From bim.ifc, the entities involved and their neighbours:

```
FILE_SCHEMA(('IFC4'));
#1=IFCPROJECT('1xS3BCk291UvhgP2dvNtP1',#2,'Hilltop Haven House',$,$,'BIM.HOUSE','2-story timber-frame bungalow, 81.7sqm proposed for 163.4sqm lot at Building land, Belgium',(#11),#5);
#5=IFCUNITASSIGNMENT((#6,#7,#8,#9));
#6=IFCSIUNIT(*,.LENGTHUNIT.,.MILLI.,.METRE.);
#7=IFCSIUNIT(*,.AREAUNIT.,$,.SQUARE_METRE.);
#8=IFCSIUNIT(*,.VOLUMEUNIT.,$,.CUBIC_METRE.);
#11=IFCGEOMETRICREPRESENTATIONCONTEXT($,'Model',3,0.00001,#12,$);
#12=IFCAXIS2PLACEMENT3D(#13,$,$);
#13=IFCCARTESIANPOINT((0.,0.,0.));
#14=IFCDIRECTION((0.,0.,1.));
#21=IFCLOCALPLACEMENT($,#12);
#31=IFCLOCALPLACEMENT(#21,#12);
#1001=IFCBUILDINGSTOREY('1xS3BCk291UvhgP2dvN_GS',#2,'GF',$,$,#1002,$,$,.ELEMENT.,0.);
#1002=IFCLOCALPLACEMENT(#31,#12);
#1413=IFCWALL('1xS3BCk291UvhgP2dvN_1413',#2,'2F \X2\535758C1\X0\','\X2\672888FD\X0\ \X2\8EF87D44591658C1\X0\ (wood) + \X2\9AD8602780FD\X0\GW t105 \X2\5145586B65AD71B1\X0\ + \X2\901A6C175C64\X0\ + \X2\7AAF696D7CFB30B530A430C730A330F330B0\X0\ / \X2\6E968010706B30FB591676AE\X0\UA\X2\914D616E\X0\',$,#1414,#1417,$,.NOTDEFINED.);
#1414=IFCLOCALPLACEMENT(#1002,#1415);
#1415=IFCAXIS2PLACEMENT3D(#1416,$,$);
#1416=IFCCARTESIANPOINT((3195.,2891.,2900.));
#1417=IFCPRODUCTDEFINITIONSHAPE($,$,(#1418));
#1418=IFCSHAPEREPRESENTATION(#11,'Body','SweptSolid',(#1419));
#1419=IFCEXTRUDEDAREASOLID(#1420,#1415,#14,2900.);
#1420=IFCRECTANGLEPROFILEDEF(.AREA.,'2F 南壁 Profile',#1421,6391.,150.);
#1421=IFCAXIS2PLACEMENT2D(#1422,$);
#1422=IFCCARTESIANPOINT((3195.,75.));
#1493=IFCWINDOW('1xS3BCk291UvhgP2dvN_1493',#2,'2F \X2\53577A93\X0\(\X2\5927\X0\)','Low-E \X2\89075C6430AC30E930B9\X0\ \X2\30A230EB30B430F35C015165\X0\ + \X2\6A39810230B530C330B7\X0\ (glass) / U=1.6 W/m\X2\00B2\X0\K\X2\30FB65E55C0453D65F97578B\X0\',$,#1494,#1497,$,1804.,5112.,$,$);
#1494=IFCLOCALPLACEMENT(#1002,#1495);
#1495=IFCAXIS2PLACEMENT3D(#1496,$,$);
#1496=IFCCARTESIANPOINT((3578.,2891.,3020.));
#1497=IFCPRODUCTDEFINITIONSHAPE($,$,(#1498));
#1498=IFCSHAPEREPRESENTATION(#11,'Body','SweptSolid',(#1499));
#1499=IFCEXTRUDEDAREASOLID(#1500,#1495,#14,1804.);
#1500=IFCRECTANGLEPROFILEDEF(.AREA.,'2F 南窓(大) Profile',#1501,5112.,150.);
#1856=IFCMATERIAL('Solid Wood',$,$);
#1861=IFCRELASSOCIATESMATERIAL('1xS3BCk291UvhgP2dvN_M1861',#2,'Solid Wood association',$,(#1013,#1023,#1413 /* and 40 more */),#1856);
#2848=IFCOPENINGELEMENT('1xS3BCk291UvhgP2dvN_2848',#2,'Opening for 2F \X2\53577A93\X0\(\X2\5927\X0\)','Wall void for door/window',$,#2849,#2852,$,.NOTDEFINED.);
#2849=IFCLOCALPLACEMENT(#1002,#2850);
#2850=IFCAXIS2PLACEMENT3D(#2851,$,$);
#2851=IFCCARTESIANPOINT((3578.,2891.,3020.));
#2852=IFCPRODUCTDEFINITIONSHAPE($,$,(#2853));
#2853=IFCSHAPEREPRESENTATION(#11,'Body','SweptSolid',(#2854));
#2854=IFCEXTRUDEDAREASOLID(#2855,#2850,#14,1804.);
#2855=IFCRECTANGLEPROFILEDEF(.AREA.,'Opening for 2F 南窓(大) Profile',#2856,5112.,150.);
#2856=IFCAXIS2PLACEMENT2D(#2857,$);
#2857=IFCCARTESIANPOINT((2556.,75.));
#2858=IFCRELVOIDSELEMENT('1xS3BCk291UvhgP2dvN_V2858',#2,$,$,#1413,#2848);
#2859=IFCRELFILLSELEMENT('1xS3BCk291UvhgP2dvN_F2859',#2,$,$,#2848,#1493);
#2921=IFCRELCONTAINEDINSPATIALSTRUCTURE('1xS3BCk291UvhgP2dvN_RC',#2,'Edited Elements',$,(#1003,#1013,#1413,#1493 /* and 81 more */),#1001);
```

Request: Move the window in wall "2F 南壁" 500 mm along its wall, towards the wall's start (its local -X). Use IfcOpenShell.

```python
import ifcopenshell
import ifcopenshell.api.geometry
import ifcopenshell.util.placement

model = ifcopenshell.open("bim.ifc")

window = model.by_guid("1xS3BCk291UvhgP2dvN_1493")
opening = window.FillsVoids[0].RelatingOpeningElement
wall = opening.VoidsElements[0].RelatingBuildingElement

wall_matrix = ifcopenshell.util.placement.get_local_placement(wall.ObjectPlacement)
shift = wall_matrix[:3, 0] * -500.0
before = ifcopenshell.util.placement.get_local_placement(window.ObjectPlacement)[:3, 3].copy()

# The window is not placed relative to its opening, so move both.
for product in (opening, window):
    matrix = ifcopenshell.util.placement.get_local_placement(product.ObjectPlacement)
    matrix[:3, 3] += shift
    ifcopenshell.api.geometry.edit_object_placement(model, product=product, matrix=matrix, is_si=False)

after = ifcopenshell.util.placement.get_local_placement(window.ObjectPlacement)[:3, 3]
print("window moved by", (after - before).round(3) + 0.0)

model.write("bim-out.ifc")
```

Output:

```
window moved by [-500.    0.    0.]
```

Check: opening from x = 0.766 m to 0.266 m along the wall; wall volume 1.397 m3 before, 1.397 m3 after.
